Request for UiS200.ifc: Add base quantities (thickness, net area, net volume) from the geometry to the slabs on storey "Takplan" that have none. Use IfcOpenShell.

First a look at what the model holds.

```python
import ifcopenshell
import ifcopenshell.util.element
import ifcopenshell.util.unit

model = ifcopenshell.open("UiS200.ifc")
print(model.schema)
for unit_type in ("LENGTHUNIT", "AREAUNIT", "VOLUMEUNIT"):
    print(unit_type, ifcopenshell.util.unit.calculate_unit_scale(model, unit_type))
storey = next(s for s in model.by_type("IfcBuildingStorey") if s.Name == "Takplan")
slabs = [e for e in ifcopenshell.util.element.get_decomposition(storey) if e.is_a("IfcSlab")]
for e in sorted(slabs, key=lambda e: e.id()):
    print(e.id(), e.is_a(), e.Name, list(ifcopenshell.util.element.get_psets(e, qtos_only=True)), sep=" | ")
```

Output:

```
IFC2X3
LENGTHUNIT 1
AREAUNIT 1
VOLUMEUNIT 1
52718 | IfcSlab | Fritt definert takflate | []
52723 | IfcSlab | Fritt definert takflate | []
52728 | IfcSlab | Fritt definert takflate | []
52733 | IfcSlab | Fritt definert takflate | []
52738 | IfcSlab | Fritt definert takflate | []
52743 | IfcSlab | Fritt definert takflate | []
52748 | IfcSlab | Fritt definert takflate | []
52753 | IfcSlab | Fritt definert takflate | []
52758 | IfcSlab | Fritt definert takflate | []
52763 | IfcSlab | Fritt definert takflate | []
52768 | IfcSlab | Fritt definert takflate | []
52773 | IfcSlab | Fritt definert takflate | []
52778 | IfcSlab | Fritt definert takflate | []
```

```python
import ifcopenshell
import ifcopenshell.api.pset
import ifcopenshell.geom
import ifcopenshell.util.element
import ifcopenshell.util.shape
import ifcopenshell.util.unit

model = ifcopenshell.open("UiS200.ifc")
unit_scale = ifcopenshell.util.unit.calculate_unit_scale(model)
area_scale = ifcopenshell.util.unit.calculate_unit_scale(model, "AREAUNIT")
volume_scale = ifcopenshell.util.unit.calculate_unit_scale(model, "VOLUMEUNIT")
settings = ifcopenshell.geom.settings()

storey = next(s for s in model.by_type("IfcBuildingStorey") if s.Name == "Takplan")
slabs = [e for e in ifcopenshell.util.element.get_decomposition(storey) if e.is_a("IfcSlab")]

for e in sorted(slabs, key=lambda e: e.id()):
    if ifcopenshell.util.element.get_psets(e, qtos_only=True, should_inherit=False):
        continue
    # Geometry comes back in metres, in the element's own axes.
    shape = ifcopenshell.geom.create_shape(settings, e)
    values = {
        "Width": ifcopenshell.util.shape.get_z(shape.geometry) / unit_scale,
        "NetArea": ifcopenshell.util.shape.get_footprint_area(shape.geometry) / area_scale,
        "NetVolume": ifcopenshell.util.shape.get_volume(shape.geometry) / volume_scale,
    }
    qto = ifcopenshell.api.pset.add_qto(model, product=e, name="BaseQuantities")
    ifcopenshell.api.pset.edit_qto(model, qto=qto, properties=values)
    print(e.id(), {k: round(v, 3) for k, v in values.items()})

model.write("UiS200-out.ifc")
```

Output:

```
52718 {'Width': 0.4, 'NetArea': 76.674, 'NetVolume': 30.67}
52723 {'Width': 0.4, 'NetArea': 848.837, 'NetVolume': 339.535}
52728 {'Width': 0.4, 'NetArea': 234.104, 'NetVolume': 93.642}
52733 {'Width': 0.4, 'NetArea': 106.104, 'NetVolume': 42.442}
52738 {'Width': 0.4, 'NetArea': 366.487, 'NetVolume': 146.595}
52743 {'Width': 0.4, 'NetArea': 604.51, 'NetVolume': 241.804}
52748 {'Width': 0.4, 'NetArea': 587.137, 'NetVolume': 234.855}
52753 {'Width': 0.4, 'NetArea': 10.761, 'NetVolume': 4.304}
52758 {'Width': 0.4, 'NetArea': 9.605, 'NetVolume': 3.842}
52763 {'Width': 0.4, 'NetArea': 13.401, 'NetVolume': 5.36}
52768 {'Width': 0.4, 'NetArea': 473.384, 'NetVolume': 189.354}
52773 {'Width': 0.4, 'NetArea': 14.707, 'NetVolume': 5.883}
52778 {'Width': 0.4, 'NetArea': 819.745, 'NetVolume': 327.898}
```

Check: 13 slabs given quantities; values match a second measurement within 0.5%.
